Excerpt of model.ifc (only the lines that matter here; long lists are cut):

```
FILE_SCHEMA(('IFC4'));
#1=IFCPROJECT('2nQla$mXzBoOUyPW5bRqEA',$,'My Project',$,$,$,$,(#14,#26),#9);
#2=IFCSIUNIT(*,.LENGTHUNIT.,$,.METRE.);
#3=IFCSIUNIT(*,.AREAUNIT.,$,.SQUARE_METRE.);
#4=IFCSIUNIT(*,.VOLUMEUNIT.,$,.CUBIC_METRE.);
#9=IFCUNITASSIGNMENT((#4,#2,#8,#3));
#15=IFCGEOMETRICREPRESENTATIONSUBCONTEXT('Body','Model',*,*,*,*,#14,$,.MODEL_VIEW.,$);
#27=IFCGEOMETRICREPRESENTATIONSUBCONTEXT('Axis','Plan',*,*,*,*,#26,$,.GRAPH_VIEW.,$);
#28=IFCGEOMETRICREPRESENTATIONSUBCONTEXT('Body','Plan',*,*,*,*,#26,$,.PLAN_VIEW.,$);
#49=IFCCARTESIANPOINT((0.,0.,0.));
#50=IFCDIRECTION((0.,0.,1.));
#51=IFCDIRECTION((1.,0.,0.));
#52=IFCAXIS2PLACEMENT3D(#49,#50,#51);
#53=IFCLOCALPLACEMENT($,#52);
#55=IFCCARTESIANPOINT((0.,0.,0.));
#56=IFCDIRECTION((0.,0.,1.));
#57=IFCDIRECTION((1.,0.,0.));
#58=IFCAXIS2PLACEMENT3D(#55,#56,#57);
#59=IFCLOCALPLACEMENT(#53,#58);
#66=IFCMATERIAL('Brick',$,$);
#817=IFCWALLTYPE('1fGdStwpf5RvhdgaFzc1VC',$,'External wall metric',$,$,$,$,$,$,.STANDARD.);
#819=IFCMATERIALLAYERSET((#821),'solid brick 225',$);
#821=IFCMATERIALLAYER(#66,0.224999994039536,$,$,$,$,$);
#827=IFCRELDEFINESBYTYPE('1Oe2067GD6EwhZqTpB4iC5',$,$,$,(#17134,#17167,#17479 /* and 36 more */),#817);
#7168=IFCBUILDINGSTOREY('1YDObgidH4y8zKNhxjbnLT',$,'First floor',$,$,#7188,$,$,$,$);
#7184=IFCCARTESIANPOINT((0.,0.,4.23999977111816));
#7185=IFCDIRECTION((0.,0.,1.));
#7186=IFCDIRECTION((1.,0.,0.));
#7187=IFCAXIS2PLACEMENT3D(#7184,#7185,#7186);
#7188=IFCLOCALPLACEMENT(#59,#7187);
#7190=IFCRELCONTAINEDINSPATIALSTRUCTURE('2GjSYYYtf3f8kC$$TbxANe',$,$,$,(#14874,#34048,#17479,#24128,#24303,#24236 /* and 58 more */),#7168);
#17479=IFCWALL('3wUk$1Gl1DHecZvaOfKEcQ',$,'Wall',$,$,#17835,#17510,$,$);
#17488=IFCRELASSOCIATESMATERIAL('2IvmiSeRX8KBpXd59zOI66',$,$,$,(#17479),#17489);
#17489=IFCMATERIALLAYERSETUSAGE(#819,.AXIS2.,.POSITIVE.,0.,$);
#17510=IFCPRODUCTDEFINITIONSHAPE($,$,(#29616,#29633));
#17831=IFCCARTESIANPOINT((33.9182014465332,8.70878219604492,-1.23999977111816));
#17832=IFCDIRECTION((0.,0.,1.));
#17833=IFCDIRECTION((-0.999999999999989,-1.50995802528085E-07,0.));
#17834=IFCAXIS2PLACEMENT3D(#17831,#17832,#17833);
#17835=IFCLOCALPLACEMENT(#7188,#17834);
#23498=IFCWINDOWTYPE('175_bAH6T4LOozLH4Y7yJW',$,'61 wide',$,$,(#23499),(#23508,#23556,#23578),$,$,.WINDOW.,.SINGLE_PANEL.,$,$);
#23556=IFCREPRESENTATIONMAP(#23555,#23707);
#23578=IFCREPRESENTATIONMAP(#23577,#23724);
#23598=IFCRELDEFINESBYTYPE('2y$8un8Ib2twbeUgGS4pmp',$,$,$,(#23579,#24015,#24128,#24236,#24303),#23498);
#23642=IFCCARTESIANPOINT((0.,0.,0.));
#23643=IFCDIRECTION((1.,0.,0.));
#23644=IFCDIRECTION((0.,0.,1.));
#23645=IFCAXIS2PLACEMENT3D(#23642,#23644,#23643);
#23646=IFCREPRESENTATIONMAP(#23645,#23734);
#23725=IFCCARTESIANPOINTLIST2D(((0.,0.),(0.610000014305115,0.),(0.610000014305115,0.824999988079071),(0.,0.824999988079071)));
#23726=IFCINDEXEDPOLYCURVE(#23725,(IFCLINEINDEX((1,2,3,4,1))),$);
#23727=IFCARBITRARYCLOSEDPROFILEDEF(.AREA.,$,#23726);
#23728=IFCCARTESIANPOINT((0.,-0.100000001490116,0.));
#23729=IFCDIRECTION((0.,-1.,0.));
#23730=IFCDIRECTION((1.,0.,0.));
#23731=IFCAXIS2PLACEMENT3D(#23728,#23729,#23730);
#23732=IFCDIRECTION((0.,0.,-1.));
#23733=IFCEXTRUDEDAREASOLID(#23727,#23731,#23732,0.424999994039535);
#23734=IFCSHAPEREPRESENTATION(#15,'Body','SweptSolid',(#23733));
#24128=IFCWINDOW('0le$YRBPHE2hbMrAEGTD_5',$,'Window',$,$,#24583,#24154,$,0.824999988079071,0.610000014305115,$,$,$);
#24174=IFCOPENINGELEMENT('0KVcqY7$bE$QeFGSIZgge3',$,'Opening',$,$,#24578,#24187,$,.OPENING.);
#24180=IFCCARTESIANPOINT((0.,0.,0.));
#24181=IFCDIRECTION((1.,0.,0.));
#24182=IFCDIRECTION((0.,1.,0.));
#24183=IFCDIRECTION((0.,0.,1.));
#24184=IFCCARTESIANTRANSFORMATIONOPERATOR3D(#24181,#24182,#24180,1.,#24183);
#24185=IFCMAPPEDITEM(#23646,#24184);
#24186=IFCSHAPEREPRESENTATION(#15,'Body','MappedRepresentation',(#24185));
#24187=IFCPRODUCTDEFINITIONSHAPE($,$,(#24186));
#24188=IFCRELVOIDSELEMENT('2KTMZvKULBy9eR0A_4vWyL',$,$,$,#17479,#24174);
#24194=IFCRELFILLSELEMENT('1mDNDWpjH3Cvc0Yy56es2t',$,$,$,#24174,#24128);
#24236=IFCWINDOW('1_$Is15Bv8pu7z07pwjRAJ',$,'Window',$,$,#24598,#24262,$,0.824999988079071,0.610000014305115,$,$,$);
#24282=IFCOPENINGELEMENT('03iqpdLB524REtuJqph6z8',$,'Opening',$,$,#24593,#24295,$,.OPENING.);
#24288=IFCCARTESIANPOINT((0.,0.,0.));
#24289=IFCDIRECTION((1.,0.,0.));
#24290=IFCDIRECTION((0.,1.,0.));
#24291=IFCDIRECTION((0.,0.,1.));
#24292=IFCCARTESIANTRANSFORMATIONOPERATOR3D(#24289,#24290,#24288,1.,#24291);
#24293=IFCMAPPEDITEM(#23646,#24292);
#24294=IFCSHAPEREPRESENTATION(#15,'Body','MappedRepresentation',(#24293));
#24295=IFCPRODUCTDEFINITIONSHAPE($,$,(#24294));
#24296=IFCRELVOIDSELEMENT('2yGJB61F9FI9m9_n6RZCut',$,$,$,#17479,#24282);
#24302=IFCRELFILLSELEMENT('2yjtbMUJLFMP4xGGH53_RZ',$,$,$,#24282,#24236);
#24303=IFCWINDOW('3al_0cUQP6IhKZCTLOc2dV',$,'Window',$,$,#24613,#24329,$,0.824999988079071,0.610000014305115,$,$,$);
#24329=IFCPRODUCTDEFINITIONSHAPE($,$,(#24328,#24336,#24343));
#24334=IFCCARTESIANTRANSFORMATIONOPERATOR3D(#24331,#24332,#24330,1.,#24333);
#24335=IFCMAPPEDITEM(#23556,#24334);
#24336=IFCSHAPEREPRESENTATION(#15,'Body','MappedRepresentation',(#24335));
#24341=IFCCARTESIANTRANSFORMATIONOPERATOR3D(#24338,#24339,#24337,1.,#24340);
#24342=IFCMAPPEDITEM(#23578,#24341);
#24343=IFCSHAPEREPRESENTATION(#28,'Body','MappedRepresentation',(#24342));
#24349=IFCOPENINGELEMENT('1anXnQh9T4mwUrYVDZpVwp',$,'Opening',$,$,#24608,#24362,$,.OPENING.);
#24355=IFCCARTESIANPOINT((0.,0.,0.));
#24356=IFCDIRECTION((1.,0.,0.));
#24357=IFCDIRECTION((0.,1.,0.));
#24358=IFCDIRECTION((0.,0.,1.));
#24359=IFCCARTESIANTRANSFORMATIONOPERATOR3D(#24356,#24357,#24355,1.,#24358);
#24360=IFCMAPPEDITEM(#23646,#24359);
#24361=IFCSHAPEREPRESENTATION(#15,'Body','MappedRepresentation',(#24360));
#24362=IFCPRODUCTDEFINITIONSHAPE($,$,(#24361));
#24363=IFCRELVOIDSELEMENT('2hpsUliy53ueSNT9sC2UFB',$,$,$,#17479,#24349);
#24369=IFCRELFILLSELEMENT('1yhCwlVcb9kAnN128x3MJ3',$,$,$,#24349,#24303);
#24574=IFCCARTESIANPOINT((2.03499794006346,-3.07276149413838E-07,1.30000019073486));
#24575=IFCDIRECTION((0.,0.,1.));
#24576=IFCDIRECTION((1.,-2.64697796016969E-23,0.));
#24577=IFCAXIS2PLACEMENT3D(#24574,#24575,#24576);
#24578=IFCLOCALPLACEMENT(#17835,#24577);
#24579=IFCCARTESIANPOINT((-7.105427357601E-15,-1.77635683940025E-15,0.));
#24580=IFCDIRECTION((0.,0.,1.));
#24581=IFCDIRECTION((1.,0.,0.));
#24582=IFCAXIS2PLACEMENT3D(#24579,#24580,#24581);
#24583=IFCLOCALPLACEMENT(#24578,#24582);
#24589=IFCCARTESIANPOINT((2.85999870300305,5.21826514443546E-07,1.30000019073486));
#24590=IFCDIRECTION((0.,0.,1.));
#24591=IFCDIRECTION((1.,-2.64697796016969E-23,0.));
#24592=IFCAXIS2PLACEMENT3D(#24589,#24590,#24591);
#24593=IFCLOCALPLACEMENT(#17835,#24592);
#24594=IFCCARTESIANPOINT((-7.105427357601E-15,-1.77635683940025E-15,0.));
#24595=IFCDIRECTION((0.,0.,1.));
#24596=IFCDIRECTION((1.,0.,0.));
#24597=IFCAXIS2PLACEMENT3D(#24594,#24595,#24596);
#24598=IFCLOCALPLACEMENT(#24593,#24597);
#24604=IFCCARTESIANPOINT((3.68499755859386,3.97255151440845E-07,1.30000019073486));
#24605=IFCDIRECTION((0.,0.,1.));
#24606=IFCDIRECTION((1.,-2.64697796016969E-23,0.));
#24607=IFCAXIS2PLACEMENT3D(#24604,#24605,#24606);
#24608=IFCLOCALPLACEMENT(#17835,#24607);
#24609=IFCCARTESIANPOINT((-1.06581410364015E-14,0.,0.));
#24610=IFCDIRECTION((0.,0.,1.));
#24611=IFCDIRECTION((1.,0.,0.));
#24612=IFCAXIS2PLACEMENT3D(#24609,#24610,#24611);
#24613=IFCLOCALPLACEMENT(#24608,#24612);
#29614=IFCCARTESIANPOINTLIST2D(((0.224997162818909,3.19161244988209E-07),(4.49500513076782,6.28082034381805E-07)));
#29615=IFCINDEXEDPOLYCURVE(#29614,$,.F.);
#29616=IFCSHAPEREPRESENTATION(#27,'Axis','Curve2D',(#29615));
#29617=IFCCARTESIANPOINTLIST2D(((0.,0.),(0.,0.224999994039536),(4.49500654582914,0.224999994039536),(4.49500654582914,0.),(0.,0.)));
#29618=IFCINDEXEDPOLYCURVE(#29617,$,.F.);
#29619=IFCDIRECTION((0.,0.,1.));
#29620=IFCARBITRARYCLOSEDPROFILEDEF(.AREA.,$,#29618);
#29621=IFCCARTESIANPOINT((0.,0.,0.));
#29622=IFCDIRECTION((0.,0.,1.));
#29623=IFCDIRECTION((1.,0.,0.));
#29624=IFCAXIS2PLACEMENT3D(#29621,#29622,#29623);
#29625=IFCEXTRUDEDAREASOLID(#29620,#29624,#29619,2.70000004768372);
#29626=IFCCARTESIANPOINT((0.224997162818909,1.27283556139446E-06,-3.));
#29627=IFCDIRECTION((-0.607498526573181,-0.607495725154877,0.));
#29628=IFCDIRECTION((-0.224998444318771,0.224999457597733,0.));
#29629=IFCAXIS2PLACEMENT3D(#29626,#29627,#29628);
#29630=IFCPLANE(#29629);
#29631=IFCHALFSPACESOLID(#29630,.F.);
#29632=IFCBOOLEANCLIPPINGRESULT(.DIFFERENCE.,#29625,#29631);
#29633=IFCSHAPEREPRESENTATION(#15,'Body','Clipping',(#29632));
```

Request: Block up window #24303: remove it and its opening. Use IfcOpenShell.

```python
import ifcopenshell
import ifcopenshell.api.feature
import ifcopenshell.api.root
import ifcopenshell.geom
import ifcopenshell.util.shape

model = ifcopenshell.open("model.ifc")
settings = ifcopenshell.geom.settings()


def volume(element):
    """Net volume in cubic metres, openings subtracted."""
    shape = ifcopenshell.geom.create_shape(settings, element)
    return ifcopenshell.util.shape.get_volume(shape.geometry)


window = model.by_guid("3al_0cUQP6IhKZCTLOc2dV")
opening = window.FillsVoids[0].RelatingOpeningElement
wall = opening.VoidsElements[0].RelatingBuildingElement
before = volume(wall)

ifcopenshell.api.root.remove_product(model, product=window)
ifcopenshell.api.feature.remove_feature(model, feature=opening)

after = volume(wall)

print(f"wall volume {before:.3f} -> {after:.3f} m3")

model.write("model-out.ifc")
```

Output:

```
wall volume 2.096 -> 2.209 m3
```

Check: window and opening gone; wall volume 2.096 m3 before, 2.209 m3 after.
